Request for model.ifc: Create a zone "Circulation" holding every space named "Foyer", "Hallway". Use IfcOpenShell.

First a look at what the model holds.

```python
import ifcopenshell

model = ifcopenshell.open("model.ifc")
print(model.schema)
seen = {}
for space in model.by_type("IfcSpace"):
    seen[space.LongName] = seen.get(space.LongName, 0) + 1
for name, count in sorted(seen.items(), key=str):
    print(count, "x", name)
print("zones:", [z.Name for z in model.by_type("IfcZone")][:20])
```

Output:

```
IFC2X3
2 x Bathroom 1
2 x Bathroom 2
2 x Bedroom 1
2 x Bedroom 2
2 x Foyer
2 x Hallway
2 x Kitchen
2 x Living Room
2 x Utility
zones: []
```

```python
import ifcopenshell
import ifcopenshell.api.group
import ifcopenshell.api.root

model = ifcopenshell.open("model.ifc")

names = {"Foyer", "Hallway"}
spaces = [s for s in model.by_type("IfcSpace") if s.LongName in names]

zone = ifcopenshell.api.root.create_entity(model, ifc_class="IfcZone", name="Circulation")
ifcopenshell.api.group.assign_group(model, products=spaces, group=zone)
print(len(spaces), "spaces in", zone.Name)

model.write("model_updated.ifc")
```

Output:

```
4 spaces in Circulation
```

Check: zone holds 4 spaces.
